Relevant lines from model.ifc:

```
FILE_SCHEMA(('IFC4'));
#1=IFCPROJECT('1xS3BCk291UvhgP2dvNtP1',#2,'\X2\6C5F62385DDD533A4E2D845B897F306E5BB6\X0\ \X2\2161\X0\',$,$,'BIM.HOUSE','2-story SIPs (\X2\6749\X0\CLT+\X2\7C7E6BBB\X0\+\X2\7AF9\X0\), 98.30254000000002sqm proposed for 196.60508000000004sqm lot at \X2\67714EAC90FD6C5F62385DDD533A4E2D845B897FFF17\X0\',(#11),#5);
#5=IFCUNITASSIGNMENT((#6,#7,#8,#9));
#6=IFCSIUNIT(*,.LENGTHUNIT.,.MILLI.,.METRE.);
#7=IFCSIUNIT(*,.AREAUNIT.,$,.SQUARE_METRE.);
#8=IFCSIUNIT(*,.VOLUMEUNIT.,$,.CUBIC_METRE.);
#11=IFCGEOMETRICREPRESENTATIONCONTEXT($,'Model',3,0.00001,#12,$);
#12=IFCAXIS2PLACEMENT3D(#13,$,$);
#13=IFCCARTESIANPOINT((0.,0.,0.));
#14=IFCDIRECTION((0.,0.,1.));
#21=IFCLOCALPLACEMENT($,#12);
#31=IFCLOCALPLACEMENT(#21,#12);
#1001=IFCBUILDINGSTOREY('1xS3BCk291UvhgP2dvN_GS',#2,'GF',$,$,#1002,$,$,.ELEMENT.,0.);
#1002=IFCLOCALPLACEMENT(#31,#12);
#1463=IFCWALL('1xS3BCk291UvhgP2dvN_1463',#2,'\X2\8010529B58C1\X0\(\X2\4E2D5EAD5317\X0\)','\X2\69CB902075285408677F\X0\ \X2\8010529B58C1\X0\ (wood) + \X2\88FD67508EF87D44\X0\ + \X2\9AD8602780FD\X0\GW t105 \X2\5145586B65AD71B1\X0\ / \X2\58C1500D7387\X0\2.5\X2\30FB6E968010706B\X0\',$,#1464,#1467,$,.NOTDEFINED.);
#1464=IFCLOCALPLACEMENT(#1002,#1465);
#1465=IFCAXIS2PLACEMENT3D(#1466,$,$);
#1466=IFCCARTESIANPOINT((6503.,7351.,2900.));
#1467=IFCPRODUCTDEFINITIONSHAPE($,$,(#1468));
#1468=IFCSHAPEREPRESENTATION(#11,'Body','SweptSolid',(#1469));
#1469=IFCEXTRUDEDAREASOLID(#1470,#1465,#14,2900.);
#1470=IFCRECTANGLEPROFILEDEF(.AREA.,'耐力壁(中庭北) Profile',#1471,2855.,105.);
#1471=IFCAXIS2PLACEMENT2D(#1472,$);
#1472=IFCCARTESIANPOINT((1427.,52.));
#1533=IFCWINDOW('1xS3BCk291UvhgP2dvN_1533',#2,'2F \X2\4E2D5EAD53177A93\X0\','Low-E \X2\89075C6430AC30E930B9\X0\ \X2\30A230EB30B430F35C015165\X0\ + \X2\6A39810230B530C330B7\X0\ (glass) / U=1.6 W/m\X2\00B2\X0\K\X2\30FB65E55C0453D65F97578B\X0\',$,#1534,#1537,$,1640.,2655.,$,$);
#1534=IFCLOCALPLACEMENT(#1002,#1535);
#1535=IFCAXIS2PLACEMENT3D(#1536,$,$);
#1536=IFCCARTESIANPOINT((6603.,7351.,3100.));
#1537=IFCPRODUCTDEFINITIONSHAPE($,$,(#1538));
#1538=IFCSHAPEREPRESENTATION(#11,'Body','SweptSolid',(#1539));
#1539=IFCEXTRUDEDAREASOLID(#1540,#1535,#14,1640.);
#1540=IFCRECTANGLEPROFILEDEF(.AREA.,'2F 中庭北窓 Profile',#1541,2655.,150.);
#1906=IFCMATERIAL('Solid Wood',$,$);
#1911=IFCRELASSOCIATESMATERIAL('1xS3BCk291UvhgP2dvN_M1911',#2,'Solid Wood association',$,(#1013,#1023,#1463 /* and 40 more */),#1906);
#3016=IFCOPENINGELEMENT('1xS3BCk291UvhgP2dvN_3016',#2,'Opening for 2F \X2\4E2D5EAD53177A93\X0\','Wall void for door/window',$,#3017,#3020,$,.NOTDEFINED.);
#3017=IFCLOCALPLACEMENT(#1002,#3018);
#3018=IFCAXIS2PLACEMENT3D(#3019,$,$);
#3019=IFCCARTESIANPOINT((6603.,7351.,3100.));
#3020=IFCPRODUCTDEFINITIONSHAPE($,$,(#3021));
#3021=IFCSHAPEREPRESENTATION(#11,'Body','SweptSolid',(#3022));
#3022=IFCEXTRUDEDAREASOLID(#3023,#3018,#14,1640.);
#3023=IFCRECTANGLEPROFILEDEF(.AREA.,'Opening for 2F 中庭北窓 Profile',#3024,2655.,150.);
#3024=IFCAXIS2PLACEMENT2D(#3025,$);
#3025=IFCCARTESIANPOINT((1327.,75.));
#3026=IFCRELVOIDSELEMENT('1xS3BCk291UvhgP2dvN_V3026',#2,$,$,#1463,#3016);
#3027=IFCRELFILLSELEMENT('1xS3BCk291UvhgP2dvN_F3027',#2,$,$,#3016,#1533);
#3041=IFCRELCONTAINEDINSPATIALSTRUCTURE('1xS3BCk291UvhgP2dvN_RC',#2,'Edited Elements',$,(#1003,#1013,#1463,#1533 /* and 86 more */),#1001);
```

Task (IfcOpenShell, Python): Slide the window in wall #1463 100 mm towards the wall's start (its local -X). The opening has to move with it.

```python
import ifcopenshell
import ifcopenshell.api.geometry
import ifcopenshell.util.placement
import ifcopenshell.util.unit

model = ifcopenshell.open("model.ifc")
unit_scale = ifcopenshell.util.unit.calculate_unit_scale(model)

window = model.by_guid("1xS3BCk291UvhgP2dvN_1533")
opening = window.FillsVoids[0].RelatingOpeningElement
wall = opening.VoidsElements[0].RelatingBuildingElement

wall_matrix = ifcopenshell.util.placement.get_local_placement(wall.ObjectPlacement)
shift = wall_matrix[:3, 0] * -0.1 / unit_scale
before = ifcopenshell.util.placement.get_local_placement(window.ObjectPlacement)[:3, 3].copy()

# The window is not placed relative to its opening, so move both.
for product in (opening, window):
    matrix = ifcopenshell.util.placement.get_local_placement(product.ObjectPlacement)
    matrix[:3, 3] += shift
    ifcopenshell.api.geometry.edit_object_placement(model, product=product, matrix=matrix, is_si=False)

after = ifcopenshell.util.placement.get_local_placement(window.ObjectPlacement)[:3, 3]
print("window moved by", (after - before).round(3) + 0.0)

model.write("model_edited.ifc")
```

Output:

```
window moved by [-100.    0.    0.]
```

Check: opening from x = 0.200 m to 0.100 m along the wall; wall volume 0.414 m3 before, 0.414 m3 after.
